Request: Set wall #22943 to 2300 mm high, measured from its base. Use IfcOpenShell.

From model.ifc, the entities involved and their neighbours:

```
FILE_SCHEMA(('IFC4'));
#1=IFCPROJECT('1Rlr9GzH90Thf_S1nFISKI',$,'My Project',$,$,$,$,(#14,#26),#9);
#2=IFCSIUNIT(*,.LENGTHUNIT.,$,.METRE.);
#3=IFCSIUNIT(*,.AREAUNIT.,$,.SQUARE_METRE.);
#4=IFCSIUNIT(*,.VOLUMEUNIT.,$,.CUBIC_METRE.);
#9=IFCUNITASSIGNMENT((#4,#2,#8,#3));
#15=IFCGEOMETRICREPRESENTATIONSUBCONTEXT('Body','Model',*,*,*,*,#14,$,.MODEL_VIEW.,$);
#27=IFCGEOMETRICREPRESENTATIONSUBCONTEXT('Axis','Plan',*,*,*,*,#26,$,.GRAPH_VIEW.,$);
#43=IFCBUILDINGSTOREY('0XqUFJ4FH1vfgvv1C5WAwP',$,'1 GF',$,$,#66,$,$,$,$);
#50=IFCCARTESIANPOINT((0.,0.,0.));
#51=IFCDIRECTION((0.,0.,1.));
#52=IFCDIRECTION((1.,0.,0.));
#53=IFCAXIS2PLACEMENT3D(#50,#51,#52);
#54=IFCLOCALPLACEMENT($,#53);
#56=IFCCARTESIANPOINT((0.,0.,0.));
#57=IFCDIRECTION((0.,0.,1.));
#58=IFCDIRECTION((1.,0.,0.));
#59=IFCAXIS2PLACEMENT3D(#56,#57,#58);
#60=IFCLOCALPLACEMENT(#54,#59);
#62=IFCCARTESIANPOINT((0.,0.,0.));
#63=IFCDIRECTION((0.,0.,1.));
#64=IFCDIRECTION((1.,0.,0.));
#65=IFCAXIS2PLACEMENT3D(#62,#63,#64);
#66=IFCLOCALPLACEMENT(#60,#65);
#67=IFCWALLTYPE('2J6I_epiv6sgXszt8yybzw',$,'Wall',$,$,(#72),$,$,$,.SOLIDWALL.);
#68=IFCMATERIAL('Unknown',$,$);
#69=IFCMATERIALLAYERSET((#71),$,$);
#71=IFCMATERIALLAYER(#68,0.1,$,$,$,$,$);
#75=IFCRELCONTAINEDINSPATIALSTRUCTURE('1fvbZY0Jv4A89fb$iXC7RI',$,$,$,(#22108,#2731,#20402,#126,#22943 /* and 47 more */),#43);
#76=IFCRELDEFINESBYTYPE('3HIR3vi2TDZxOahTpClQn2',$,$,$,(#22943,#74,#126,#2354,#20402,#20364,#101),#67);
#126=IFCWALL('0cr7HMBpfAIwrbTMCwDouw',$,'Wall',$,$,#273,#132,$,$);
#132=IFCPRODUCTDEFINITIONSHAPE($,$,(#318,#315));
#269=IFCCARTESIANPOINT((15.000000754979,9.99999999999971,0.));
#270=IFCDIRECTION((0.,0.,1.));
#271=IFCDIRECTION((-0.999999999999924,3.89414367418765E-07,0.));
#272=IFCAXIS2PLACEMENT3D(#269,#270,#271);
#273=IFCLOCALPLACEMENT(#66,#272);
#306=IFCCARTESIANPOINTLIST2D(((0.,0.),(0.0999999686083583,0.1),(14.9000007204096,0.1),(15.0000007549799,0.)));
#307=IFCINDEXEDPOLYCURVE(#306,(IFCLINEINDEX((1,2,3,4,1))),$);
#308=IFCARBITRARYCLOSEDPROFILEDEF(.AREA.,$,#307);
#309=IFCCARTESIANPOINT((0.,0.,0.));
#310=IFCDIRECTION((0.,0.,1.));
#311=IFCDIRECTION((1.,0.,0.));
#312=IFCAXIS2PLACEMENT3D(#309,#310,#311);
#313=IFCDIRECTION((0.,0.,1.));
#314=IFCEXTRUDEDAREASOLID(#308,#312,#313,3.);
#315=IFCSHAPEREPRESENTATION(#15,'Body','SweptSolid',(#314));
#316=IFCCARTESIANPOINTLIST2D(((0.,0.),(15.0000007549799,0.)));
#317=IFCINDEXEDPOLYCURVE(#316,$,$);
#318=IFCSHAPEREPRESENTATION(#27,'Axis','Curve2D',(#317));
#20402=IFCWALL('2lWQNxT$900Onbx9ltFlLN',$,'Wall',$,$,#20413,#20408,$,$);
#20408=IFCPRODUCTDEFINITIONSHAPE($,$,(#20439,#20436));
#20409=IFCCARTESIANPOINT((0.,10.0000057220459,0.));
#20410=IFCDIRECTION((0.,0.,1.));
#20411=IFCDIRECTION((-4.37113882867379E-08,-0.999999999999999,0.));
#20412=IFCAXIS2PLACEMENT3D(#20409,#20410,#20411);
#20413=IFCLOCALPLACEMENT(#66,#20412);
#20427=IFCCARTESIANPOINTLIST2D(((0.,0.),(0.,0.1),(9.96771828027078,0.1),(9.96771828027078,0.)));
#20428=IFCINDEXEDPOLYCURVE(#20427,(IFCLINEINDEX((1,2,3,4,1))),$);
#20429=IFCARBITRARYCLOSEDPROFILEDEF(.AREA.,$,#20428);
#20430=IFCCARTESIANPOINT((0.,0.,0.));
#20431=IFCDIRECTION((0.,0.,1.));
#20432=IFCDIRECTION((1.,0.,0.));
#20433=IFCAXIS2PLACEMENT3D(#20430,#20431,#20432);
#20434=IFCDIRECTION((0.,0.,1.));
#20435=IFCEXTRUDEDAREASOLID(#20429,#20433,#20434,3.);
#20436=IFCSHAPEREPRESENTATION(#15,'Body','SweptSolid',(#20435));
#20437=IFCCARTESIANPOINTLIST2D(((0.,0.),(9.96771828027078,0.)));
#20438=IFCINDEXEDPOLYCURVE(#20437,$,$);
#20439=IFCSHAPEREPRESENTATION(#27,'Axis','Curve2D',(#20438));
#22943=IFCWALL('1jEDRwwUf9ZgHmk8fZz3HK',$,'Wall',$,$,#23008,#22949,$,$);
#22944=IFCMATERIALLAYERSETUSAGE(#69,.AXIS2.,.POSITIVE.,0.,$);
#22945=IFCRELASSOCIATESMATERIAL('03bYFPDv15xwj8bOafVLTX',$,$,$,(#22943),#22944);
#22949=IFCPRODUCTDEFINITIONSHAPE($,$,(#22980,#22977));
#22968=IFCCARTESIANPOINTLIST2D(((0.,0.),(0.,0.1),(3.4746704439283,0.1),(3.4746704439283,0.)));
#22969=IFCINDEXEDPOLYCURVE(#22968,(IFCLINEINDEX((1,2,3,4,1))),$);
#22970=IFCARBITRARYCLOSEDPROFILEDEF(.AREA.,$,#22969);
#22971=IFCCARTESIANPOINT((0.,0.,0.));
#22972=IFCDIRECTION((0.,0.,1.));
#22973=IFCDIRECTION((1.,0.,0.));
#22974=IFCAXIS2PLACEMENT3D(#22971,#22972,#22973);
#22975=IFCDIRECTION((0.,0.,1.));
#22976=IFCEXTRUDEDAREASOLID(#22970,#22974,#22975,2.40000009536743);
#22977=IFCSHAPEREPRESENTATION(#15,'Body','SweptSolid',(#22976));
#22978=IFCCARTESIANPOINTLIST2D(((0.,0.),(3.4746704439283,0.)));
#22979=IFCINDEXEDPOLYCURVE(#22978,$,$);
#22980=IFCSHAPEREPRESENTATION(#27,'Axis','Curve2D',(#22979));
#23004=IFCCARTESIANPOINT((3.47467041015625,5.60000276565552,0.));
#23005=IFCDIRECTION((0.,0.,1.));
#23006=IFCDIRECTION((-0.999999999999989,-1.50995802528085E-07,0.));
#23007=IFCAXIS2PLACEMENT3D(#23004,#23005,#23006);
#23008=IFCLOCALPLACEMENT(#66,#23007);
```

```python
import ifcopenshell
import ifcopenshell.geom
import ifcopenshell.util.representation
import ifcopenshell.util.shape

model = ifcopenshell.open("model.ifc")
settings = ifcopenshell.geom.settings()


def volume(element):
    """Net volume in cubic metres, openings subtracted."""
    shape = ifcopenshell.geom.create_shape(settings, element)
    return ifcopenshell.util.shape.get_volume(shape.geometry)


wall = model.by_guid("1jEDRwwUf9ZgHmk8fZz3HK")
before = volume(wall)

body = ifcopenshell.util.representation.get_representation(wall, "Model", "Body")
solid = body.Items[0]
old_height = solid.Depth
solid.Depth = 2.3
after = volume(wall)

print(f"height {old_height:g} -> {solid.Depth:g}, volume {before:.3f} -> {after:.3f} m3")

model.write("model-out.ifc")
```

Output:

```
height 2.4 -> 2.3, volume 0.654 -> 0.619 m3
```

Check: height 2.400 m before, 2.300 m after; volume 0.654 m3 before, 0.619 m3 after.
